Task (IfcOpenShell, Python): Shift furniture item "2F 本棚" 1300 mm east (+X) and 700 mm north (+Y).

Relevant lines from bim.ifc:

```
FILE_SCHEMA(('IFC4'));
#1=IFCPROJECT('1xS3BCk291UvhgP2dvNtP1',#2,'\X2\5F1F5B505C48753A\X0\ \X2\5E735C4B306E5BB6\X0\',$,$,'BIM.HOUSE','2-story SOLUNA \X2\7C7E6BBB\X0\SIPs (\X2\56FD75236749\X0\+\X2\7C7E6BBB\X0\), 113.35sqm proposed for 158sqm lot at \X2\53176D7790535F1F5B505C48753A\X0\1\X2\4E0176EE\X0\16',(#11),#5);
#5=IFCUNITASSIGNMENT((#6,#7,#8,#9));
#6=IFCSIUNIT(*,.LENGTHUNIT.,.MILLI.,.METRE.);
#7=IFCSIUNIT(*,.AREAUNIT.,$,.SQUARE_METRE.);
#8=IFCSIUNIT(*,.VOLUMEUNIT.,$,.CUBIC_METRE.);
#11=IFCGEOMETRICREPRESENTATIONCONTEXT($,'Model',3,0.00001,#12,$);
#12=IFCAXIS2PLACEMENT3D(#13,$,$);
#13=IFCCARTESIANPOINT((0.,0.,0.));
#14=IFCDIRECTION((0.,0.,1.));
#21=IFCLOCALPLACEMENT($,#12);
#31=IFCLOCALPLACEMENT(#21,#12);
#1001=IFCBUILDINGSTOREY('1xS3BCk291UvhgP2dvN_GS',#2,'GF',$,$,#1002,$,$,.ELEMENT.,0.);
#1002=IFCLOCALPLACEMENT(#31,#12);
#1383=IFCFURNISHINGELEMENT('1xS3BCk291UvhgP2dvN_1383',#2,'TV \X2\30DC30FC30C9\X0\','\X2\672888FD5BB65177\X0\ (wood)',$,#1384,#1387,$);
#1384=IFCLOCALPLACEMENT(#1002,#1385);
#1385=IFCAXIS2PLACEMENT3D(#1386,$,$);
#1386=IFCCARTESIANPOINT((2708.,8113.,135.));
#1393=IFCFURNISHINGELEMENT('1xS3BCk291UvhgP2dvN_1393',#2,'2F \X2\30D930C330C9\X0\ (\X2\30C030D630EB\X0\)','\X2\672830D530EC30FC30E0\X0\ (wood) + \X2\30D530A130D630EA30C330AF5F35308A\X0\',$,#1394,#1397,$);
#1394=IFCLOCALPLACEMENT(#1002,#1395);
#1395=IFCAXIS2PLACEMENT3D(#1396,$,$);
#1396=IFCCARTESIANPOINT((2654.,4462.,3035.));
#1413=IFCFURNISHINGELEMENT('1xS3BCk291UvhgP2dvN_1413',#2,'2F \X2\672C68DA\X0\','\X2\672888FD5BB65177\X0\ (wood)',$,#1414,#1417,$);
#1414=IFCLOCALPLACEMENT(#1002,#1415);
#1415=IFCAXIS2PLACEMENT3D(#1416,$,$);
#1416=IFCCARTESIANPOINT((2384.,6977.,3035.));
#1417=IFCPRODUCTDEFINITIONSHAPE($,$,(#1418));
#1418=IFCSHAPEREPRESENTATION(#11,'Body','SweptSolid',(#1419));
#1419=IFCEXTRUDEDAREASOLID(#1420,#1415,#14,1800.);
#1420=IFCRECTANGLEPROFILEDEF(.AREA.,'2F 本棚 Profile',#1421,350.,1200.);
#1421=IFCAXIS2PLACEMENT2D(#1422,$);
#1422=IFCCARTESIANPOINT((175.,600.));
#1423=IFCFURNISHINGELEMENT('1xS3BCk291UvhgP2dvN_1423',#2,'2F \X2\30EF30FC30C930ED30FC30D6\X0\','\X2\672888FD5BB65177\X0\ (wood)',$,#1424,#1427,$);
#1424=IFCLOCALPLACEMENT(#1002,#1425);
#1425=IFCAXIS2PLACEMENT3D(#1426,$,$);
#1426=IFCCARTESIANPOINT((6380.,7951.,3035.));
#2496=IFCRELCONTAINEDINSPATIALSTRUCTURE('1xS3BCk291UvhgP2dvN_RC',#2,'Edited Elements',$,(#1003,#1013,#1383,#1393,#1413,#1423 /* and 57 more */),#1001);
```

```python
import ifcopenshell
import ifcopenshell.api.geometry
import ifcopenshell.util.placement

model = ifcopenshell.open("bim.ifc")

item = model.by_id(1413)
matrix = ifcopenshell.util.placement.get_local_placement(item.ObjectPlacement)
matrix[0, 3] += 1300.0
matrix[1, 3] += 700.0
ifcopenshell.api.geometry.edit_object_placement(model, product=item, matrix=matrix, is_si=False)

print(ifcopenshell.util.placement.get_local_placement(item.ObjectPlacement).round(3) + 0.0)

model.write("bim_v2.ifc")
```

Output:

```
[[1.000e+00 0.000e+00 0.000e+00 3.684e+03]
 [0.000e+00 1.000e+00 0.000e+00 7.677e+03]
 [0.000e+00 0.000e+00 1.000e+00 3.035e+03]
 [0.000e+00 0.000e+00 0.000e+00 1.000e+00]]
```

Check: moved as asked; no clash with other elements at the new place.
